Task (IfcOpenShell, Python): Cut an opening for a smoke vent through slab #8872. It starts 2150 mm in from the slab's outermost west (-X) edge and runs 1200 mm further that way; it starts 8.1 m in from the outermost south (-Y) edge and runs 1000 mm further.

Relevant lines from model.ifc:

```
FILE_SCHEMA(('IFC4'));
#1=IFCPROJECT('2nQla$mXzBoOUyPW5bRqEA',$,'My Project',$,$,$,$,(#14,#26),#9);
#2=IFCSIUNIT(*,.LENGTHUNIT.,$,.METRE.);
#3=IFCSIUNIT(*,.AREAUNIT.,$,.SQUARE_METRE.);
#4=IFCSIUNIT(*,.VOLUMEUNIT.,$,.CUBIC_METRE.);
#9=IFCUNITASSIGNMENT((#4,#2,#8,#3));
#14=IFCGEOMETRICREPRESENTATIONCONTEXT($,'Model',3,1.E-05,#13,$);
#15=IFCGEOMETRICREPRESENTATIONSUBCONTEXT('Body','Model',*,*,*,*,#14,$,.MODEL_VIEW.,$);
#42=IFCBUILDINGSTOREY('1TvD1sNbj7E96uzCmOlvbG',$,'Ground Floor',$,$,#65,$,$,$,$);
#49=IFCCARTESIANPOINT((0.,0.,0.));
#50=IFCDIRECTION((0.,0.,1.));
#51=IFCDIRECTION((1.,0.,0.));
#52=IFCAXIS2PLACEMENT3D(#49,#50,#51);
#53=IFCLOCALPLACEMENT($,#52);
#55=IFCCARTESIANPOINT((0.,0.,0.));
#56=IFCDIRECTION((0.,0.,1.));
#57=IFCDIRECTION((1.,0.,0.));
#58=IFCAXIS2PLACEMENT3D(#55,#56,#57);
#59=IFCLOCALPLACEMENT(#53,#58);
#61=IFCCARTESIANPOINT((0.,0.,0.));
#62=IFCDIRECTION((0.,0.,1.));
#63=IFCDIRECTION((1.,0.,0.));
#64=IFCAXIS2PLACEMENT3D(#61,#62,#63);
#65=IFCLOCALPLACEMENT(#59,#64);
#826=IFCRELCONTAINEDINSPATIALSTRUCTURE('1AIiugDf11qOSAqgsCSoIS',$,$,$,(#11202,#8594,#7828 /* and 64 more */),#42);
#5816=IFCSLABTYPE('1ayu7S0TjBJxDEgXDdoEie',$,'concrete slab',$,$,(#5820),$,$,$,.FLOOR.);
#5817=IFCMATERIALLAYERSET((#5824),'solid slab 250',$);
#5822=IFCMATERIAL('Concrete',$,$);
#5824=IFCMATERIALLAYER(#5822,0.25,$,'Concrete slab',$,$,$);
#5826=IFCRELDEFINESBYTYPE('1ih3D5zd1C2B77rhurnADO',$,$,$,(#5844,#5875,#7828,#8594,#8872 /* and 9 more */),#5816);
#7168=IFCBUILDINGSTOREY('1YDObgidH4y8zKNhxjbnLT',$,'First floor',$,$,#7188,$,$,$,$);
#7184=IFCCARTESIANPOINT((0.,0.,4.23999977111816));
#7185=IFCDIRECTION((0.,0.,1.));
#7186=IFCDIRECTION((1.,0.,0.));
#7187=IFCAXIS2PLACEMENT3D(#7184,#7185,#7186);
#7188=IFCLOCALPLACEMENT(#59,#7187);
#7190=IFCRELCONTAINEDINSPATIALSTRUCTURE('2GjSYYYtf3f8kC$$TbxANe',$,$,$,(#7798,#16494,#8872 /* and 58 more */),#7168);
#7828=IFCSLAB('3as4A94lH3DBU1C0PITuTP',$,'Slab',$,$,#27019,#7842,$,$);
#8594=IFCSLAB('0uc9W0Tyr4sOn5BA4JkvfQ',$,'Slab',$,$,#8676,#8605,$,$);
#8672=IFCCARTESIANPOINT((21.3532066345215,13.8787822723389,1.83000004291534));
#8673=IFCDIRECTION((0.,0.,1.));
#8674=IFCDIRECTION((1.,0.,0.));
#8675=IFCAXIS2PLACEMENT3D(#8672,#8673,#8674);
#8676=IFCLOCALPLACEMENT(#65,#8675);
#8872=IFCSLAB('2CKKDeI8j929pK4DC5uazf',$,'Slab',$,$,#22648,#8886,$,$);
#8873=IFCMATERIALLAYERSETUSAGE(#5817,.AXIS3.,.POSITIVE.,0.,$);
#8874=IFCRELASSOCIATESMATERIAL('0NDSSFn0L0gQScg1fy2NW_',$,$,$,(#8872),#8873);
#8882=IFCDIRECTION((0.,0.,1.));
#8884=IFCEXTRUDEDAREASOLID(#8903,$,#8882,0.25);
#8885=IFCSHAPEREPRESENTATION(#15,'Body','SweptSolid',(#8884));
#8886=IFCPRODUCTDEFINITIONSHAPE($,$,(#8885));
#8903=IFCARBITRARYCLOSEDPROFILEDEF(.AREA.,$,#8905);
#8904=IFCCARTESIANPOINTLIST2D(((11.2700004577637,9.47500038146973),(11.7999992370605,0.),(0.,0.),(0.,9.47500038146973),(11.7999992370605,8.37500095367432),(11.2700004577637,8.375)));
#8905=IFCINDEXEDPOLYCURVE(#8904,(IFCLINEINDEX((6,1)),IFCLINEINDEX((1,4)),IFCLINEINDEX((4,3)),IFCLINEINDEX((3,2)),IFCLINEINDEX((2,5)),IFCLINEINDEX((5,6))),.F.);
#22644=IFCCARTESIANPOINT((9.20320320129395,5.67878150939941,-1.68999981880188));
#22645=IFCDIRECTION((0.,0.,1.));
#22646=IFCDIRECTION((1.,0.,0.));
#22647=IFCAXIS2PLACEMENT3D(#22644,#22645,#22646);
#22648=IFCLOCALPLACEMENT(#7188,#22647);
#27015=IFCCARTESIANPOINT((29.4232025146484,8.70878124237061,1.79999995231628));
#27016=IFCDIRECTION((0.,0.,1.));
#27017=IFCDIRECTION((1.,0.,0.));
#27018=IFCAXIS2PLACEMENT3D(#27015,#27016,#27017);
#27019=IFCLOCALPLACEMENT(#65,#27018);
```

```python
import numpy as np
import ifcopenshell
import ifcopenshell.api.feature
import ifcopenshell.api.geometry
import ifcopenshell.api.root
import ifcopenshell.geom
import ifcopenshell.util.placement
import ifcopenshell.util.representation
import ifcopenshell.util.shape
import ifcopenshell.util.unit

model = ifcopenshell.open("model.ifc")
unit_scale = ifcopenshell.util.unit.calculate_unit_scale(model)
settings = ifcopenshell.geom.settings()


def volume(element):
    """Net volume in cubic metres, openings subtracted."""
    shape = ifcopenshell.geom.create_shape(settings, element)
    return ifcopenshell.util.shape.get_volume(shape.geometry)


slab = model.by_guid("2CKKDeI8j929pK4DC5uazf")
before = volume(slab)

# Extent in the slab's own axes, in metres. The edges named are its -X and -Y sides.
slab_shape = ifcopenshell.geom.create_shape(settings, slab)
vertices = ifcopenshell.util.shape.get_vertices(slab_shape.geometry)
x_min, y_min, bottom = vertices.min(axis=0)
top = vertices[:, 2].max()

opening = ifcopenshell.api.root.create_entity(model, ifc_class="IfcOpeningElement", name="Smoke vent opening", predefined_type="OPENING")
context = ifcopenshell.util.representation.get_context(model, "Model", "Body", "MODEL_VIEW")
width, depth = 1.2, 1
outline = [(0.0, 0.0), (width, 0.0), (width, depth), (0.0, depth), (0.0, 0.0)]
# Overshoot both faces by 50 mm so the cut is clean.
shape = ifcopenshell.api.geometry.add_slab_representation(
    model, context=context, depth=top - bottom + 0.1, polyline=outline
)
ifcopenshell.api.geometry.assign_representation(model, product=opening, representation=shape)

matrix = ifcopenshell.util.placement.get_local_placement(slab.ObjectPlacement)
matrix[:, 3] = matrix @ np.append(np.array([x_min + 2.15, y_min + 8.1, bottom - 0.05]) / unit_scale, 1.0)
ifcopenshell.api.geometry.edit_object_placement(model, product=opening, matrix=matrix, is_si=False)
ifcopenshell.api.feature.add_feature(model, feature=opening, element=slab)

after = volume(slab)

print(f"slab volume {before:.3f} -> {after:.3f} m3")

model.write("model-out.ifc")
```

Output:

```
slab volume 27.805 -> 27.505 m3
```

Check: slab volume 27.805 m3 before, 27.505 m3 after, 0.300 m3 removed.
